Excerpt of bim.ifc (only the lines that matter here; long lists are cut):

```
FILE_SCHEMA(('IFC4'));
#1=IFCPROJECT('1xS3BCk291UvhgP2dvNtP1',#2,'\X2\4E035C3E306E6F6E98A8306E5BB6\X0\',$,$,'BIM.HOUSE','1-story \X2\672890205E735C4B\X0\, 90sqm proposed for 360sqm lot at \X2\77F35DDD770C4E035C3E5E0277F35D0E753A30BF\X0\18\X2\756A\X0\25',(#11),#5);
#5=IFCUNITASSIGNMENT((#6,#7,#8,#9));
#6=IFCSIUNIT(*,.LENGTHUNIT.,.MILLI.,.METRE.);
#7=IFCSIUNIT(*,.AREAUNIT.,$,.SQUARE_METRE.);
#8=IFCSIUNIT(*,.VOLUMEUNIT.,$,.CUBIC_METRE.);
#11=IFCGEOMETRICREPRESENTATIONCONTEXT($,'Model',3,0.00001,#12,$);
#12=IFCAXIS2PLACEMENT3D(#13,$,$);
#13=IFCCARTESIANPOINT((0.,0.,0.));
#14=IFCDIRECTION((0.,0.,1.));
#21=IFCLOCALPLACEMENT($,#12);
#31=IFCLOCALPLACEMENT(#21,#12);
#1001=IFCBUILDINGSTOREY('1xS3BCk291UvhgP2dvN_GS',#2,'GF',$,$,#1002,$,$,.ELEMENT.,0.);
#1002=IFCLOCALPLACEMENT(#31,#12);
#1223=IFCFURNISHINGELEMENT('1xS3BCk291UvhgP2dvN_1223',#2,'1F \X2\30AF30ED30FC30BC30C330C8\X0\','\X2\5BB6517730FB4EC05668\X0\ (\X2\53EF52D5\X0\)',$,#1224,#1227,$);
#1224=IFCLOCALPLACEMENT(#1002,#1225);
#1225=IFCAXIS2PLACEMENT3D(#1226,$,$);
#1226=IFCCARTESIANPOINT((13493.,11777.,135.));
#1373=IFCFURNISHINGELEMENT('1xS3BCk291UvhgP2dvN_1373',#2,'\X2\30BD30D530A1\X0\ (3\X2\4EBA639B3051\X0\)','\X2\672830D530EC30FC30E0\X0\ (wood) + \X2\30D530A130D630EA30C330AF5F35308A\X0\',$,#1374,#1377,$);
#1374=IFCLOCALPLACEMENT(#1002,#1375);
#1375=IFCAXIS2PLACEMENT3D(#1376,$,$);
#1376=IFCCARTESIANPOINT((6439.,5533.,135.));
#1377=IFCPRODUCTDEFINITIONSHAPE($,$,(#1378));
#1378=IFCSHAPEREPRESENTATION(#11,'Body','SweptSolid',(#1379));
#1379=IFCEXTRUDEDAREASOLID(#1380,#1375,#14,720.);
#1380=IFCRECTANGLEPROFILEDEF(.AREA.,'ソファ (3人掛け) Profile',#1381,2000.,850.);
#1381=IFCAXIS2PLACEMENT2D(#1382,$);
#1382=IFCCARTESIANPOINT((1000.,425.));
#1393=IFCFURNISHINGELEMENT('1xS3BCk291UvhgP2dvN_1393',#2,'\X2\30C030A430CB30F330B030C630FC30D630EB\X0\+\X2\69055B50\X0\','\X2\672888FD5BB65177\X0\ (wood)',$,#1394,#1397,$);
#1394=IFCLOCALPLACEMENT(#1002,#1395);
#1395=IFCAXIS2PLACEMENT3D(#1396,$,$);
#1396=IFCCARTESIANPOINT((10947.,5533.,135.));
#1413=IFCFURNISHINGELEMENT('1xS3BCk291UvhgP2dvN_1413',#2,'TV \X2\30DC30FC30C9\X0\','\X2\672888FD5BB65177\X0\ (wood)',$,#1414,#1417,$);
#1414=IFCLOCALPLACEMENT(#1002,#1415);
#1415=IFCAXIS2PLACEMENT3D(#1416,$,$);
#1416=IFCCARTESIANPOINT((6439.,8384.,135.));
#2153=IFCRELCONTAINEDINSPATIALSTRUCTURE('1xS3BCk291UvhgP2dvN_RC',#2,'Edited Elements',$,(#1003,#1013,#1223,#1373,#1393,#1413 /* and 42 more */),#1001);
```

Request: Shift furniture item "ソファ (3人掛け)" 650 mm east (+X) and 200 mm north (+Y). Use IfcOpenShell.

```python
import ifcopenshell
import ifcopenshell.api.geometry
import ifcopenshell.util.placement

model = ifcopenshell.open("bim.ifc")

item = model.by_guid("1xS3BCk291UvhgP2dvN_1373")
matrix = ifcopenshell.util.placement.get_local_placement(item.ObjectPlacement)
matrix[0, 3] += 650.0
matrix[1, 3] += 200.0
ifcopenshell.api.geometry.edit_object_placement(model, product=item, matrix=matrix, is_si=False)

print(ifcopenshell.util.placement.get_local_placement(item.ObjectPlacement).round(3) + 0.0)

model.write("bim-out.ifc")
```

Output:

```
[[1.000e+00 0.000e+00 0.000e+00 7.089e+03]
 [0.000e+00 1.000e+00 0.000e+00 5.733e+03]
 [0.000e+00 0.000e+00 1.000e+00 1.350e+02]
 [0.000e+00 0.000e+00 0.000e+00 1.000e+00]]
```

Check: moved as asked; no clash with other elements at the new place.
